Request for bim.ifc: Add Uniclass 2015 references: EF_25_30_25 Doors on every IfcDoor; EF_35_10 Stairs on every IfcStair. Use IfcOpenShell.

First a look at what the model holds.

```python
import ifcopenshell

model = ifcopenshell.open("bim.ifc")
print(model.schema)
print("classifications:", [c.Name for c in model.by_type("IfcClassification")])
for ifc_class in ("IfcDoor", "IfcRoof", "IfcStair", "IfcWall", "IfcWindow"):
    print(ifc_class, len(model.by_type(ifc_class)))
```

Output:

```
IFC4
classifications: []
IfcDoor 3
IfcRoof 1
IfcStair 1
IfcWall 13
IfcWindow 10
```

```python
import ifcopenshell
import ifcopenshell.api.classification

model = ifcopenshell.open("bim.ifc")

system = ifcopenshell.api.classification.add_classification(model, classification="Uniclass 2015")

codes = {
    "IfcDoor": ("EF_25_30_25", "Doors"),
    "IfcStair": ("EF_35_10", "Stairs"),
}
for ifc_class, (code, name) in codes.items():
    products = model.by_type(ifc_class)
    ifcopenshell.api.classification.add_reference(
        model, products=products, classification=system, identification=code, name=name
    )
    print(code, len(products))

model.write("bim-out.ifc")
```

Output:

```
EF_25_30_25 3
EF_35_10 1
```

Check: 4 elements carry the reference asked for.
